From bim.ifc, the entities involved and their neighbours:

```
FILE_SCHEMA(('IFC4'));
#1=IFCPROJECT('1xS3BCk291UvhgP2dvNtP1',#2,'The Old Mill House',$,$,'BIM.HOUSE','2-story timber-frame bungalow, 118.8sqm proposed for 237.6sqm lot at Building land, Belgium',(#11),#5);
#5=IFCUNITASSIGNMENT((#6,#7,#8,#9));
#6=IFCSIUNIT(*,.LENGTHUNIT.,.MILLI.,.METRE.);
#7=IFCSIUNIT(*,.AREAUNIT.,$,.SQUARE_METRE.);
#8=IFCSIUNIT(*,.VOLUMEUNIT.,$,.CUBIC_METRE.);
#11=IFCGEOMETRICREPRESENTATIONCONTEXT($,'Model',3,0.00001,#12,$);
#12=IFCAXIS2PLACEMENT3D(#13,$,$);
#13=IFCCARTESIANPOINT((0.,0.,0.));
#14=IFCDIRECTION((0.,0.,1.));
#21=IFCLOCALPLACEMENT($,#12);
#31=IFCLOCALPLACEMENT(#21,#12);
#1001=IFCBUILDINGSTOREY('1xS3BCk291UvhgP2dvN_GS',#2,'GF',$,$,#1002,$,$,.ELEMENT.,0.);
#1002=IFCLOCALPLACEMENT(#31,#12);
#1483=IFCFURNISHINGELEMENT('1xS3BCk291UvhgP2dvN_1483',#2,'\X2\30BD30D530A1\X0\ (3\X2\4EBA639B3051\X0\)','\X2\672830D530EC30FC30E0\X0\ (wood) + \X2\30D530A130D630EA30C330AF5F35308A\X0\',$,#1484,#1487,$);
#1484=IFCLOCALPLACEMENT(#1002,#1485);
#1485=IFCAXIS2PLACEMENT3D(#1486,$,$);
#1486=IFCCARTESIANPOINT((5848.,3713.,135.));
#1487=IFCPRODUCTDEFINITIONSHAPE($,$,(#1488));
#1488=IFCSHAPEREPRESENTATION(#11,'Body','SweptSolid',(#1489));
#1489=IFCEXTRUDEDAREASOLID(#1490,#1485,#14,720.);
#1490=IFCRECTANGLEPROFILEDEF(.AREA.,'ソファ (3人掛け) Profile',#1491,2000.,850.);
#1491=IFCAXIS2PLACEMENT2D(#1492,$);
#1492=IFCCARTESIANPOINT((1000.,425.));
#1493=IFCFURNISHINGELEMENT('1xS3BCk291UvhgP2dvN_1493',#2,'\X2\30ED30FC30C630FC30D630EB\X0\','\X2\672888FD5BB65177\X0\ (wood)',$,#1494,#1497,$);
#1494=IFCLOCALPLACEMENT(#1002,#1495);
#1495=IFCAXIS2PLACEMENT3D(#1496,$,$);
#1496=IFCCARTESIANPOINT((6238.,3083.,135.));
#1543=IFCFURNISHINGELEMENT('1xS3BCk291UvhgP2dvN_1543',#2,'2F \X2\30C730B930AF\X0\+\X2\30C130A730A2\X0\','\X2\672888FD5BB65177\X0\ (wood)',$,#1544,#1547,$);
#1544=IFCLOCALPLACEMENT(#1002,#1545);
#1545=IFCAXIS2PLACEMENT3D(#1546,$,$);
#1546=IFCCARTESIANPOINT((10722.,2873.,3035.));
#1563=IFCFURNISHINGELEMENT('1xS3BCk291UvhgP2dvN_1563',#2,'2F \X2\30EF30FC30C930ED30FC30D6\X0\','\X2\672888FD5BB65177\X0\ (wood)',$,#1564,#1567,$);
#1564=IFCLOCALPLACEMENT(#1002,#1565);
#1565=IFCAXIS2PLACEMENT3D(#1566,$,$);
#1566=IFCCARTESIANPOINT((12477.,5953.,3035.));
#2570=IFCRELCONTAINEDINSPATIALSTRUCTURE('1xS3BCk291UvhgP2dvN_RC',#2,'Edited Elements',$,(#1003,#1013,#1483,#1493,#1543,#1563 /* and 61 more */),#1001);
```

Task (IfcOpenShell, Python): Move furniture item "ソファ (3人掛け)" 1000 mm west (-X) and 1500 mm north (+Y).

```python
import ifcopenshell
import ifcopenshell.api.geometry
import ifcopenshell.util.placement
import ifcopenshell.util.unit

model = ifcopenshell.open("bim.ifc")
unit_scale = ifcopenshell.util.unit.calculate_unit_scale(model)

item = model.by_guid("1xS3BCk291UvhgP2dvN_1483")
matrix = ifcopenshell.util.placement.get_local_placement(item.ObjectPlacement)
matrix[0, 3] -= 1 / unit_scale
matrix[1, 3] += 1.5 / unit_scale
ifcopenshell.api.geometry.edit_object_placement(model, product=item, matrix=matrix, is_si=False)

print(ifcopenshell.util.placement.get_local_placement(item.ObjectPlacement).round(3) + 0.0)

model.write("bim-out.ifc")
```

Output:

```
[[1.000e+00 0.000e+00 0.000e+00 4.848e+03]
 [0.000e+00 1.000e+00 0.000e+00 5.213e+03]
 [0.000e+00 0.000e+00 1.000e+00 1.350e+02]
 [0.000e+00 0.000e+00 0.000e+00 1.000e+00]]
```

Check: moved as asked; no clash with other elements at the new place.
